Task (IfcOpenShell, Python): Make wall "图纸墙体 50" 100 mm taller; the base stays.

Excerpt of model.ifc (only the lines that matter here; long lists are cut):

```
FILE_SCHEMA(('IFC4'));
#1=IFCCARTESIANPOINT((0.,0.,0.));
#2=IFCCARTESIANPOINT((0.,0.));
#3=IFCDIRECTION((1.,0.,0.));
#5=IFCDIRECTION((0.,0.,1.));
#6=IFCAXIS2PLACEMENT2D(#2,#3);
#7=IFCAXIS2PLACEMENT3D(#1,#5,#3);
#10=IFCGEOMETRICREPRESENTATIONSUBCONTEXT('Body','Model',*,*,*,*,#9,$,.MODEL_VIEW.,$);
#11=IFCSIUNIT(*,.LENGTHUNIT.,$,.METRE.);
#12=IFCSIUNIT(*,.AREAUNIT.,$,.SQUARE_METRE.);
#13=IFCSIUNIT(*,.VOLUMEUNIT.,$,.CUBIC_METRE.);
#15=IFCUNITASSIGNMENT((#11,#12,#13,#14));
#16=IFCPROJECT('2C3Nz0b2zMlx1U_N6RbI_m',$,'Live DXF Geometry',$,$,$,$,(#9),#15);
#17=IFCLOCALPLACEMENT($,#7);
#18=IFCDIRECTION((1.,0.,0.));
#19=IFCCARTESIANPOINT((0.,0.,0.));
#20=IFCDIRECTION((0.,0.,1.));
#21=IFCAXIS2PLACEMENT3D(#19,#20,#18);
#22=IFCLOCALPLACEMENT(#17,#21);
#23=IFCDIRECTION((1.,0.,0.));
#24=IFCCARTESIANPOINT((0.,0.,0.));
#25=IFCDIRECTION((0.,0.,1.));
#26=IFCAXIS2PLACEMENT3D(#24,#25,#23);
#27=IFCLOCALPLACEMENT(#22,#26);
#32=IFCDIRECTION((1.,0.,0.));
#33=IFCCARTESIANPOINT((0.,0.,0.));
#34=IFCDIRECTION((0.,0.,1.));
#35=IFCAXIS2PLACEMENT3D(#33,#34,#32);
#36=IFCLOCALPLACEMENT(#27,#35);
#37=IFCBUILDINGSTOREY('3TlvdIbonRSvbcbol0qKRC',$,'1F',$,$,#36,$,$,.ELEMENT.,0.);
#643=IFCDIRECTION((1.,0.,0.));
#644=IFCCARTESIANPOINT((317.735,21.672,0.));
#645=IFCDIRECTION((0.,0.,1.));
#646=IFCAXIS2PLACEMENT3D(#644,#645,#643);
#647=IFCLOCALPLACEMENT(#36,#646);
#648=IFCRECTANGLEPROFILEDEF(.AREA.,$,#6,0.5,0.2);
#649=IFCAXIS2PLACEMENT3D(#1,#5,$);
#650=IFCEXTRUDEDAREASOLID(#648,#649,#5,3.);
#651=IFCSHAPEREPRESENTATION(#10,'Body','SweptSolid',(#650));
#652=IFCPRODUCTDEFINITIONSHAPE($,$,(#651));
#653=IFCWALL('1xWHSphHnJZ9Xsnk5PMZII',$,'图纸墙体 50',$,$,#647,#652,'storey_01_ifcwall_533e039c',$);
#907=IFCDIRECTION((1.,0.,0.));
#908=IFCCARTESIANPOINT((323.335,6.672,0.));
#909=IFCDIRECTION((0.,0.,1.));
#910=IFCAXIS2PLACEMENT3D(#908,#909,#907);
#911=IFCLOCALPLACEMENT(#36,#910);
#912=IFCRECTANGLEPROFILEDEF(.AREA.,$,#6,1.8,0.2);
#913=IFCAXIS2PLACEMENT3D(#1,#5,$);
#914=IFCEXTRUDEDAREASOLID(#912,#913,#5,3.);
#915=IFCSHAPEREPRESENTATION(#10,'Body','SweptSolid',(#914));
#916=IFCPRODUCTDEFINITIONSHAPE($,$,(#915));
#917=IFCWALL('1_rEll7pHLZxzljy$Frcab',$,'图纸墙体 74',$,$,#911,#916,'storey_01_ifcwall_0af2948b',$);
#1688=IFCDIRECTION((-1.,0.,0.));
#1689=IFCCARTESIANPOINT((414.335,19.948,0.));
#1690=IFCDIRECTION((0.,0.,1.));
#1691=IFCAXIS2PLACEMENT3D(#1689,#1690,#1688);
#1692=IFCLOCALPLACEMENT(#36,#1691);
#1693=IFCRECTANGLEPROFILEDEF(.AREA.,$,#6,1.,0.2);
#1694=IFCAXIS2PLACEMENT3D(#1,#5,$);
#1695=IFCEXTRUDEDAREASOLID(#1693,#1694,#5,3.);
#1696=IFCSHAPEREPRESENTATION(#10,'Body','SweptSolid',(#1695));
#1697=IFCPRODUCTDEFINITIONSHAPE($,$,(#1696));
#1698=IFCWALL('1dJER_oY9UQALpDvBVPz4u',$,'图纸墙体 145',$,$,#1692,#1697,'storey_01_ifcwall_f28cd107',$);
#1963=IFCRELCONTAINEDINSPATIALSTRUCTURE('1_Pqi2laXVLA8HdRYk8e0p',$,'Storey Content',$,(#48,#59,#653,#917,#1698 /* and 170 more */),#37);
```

```python
import ifcopenshell
import ifcopenshell.geom
import ifcopenshell.util.representation
import ifcopenshell.util.shape

model = ifcopenshell.open("model.ifc")
settings = ifcopenshell.geom.settings()


def volume(element):
    """Net volume in cubic metres, openings subtracted."""
    shape = ifcopenshell.geom.create_shape(settings, element)
    return ifcopenshell.util.shape.get_volume(shape.geometry)


wall = model.by_id(653)
before = volume(wall)

body = ifcopenshell.util.representation.get_representation(wall, "Model", "Body")
solid = body.Items[0]
old_height = solid.Depth
solid.Depth += 0.1
after = volume(wall)

print(f"height {old_height:g} -> {solid.Depth:g}, volume {before:.3f} -> {after:.3f} m3")

model.write("model-out.ifc")
```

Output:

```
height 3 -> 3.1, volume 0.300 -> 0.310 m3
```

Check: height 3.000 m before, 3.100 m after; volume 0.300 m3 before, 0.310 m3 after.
